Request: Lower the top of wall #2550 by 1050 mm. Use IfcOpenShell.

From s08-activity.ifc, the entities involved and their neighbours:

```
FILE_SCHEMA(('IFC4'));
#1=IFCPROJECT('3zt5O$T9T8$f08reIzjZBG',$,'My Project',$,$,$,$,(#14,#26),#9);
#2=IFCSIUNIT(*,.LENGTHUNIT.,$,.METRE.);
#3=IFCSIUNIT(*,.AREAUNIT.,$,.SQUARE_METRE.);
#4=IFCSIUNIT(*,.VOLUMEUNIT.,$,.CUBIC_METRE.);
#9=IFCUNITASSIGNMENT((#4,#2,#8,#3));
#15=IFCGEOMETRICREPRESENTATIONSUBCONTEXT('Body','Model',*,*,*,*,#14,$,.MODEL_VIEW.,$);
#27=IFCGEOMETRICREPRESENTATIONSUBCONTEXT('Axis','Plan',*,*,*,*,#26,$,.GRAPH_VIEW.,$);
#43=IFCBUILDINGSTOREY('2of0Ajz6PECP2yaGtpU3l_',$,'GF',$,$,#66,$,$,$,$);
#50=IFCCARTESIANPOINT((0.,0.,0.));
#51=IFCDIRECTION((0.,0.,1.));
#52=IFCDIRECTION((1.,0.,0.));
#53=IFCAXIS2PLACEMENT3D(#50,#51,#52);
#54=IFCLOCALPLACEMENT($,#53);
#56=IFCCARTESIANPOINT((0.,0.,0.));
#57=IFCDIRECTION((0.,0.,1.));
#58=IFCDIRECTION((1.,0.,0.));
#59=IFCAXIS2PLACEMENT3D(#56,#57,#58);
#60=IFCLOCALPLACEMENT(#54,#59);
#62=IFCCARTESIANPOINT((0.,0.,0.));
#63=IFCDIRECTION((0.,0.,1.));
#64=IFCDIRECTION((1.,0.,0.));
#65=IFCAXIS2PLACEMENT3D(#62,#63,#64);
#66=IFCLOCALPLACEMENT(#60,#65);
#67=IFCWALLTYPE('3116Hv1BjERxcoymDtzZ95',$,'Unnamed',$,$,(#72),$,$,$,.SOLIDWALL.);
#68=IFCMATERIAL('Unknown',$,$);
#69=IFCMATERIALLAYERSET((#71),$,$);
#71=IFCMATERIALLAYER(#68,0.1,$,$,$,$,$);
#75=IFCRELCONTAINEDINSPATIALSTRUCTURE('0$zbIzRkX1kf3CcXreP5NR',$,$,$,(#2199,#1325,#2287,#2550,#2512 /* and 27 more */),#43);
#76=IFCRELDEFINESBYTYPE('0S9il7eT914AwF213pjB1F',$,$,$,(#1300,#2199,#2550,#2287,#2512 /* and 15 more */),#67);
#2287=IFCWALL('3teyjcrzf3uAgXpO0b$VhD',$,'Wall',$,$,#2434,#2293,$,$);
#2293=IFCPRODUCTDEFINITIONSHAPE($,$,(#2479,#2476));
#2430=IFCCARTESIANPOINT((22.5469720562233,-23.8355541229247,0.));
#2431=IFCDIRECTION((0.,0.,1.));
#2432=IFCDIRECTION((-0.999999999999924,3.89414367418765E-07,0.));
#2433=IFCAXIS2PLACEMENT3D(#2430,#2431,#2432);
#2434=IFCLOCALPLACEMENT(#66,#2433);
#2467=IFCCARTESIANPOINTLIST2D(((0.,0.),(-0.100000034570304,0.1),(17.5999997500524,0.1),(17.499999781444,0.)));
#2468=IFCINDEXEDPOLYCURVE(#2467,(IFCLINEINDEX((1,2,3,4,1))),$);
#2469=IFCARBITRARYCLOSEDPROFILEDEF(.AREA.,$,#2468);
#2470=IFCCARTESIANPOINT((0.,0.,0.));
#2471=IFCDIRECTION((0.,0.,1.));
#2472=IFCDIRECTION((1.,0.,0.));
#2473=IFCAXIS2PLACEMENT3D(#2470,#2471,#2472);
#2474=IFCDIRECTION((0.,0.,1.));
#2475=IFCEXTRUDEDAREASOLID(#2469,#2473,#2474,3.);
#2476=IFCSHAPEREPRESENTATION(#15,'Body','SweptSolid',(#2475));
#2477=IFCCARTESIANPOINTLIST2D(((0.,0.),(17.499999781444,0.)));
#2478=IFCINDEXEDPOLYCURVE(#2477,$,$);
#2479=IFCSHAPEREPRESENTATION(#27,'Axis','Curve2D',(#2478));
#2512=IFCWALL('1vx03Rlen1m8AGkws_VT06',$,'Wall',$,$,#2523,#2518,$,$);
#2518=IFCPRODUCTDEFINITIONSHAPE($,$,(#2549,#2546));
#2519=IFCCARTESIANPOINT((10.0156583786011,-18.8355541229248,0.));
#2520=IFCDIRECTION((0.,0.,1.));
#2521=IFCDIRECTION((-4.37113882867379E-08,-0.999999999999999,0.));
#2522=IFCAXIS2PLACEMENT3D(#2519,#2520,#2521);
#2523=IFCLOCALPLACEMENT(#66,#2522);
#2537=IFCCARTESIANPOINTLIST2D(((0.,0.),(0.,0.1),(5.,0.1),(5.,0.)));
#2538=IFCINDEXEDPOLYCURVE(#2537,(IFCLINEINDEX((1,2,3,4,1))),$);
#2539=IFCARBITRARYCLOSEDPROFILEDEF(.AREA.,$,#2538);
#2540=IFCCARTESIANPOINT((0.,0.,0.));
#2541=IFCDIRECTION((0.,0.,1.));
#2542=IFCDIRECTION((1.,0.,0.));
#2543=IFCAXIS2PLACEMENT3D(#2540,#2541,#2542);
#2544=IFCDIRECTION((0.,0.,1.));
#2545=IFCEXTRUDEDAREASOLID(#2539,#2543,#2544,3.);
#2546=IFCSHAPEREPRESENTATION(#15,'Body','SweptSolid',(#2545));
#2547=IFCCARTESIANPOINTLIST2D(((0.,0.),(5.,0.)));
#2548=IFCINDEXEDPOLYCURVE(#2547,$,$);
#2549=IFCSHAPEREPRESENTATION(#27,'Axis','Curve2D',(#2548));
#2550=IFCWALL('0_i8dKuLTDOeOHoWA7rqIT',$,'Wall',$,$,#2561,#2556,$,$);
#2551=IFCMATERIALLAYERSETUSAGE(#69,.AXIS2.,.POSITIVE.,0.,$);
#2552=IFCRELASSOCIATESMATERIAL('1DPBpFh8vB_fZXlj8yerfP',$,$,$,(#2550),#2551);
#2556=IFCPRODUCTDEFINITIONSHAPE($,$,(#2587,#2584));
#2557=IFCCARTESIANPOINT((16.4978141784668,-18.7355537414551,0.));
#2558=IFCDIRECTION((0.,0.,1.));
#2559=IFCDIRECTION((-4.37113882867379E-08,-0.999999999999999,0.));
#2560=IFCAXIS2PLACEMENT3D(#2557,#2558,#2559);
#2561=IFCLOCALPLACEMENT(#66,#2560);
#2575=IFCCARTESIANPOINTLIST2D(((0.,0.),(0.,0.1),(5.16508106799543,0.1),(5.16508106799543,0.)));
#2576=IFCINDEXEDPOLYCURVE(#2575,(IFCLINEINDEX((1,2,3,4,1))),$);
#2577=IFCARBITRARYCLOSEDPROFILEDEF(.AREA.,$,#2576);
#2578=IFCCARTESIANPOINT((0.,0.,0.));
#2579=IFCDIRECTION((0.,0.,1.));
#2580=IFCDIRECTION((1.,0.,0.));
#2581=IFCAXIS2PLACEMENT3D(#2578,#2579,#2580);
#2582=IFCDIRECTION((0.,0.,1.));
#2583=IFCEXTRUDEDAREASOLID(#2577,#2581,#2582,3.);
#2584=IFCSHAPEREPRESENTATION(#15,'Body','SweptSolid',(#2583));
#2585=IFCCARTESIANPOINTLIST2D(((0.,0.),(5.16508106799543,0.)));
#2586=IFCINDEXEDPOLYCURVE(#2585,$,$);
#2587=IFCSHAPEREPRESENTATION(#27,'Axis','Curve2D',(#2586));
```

```python
import ifcopenshell
import ifcopenshell.geom
import ifcopenshell.util.representation
import ifcopenshell.util.shape

model = ifcopenshell.open("s08-activity.ifc")
settings = ifcopenshell.geom.settings()


def volume(element):
    """Net volume in cubic metres, openings subtracted."""
    shape = ifcopenshell.geom.create_shape(settings, element)
    return ifcopenshell.util.shape.get_volume(shape.geometry)


wall = model.by_guid("0_i8dKuLTDOeOHoWA7rqIT")
before = volume(wall)

body = ifcopenshell.util.representation.get_representation(wall, "Model", "Body")
solid = body.Items[0]
old_height = solid.Depth
solid.Depth -= 1.05
after = volume(wall)

print(f"height {old_height:g} -> {solid.Depth:g}, volume {before:.3f} -> {after:.3f} m3")

model.write("s08-activity-out.ifc")
```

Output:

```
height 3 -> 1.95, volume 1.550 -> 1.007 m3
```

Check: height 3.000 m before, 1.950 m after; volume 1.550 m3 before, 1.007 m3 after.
